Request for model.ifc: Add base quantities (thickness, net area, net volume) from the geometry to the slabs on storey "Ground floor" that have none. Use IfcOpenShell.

First a look at what the model holds.

```python
import ifcopenshell
import ifcopenshell.util.element
import ifcopenshell.util.unit

model = ifcopenshell.open("model.ifc")
print(model.schema)
for unit_type in ("LENGTHUNIT", "AREAUNIT", "VOLUMEUNIT"):
    print(unit_type, ifcopenshell.util.unit.calculate_unit_scale(model, unit_type))
storey = next(s for s in model.by_type("IfcBuildingStorey") if s.Name == "Ground floor")
slabs = [e for e in ifcopenshell.util.element.get_decomposition(storey) if e.is_a("IfcSlab")]
for e in sorted(slabs, key=lambda e: e.id()):
    print(e.id(), e.is_a(), e.Name, list(ifcopenshell.util.element.get_psets(e, qtos_only=True)), sep=" | ")
```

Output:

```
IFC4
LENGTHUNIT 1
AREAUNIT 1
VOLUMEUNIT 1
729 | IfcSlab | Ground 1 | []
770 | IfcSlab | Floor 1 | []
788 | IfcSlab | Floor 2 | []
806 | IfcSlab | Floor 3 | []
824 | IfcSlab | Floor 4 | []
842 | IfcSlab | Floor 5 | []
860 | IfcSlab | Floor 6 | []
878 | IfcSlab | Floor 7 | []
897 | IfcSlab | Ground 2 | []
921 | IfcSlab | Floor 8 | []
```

```python
import ifcopenshell
import ifcopenshell.api.pset
import ifcopenshell.geom
import ifcopenshell.util.element
import ifcopenshell.util.shape
import ifcopenshell.util.unit

model = ifcopenshell.open("model.ifc")
unit_scale = ifcopenshell.util.unit.calculate_unit_scale(model)
area_scale = ifcopenshell.util.unit.calculate_unit_scale(model, "AREAUNIT")
volume_scale = ifcopenshell.util.unit.calculate_unit_scale(model, "VOLUMEUNIT")
settings = ifcopenshell.geom.settings()

storey = next(s for s in model.by_type("IfcBuildingStorey") if s.Name == "Ground floor")
slabs = [e for e in ifcopenshell.util.element.get_decomposition(storey) if e.is_a("IfcSlab")]

for e in sorted(slabs, key=lambda e: e.id()):
    if ifcopenshell.util.element.get_psets(e, qtos_only=True, should_inherit=False):
        continue
    # Geometry comes back in metres, in the element's own axes.
    shape = ifcopenshell.geom.create_shape(settings, e)
    values = {
        "Width": ifcopenshell.util.shape.get_z(shape.geometry) / unit_scale,
        "NetArea": ifcopenshell.util.shape.get_footprint_area(shape.geometry) / area_scale,
        "NetVolume": ifcopenshell.util.shape.get_volume(shape.geometry) / volume_scale,
    }
    qto = ifcopenshell.api.pset.add_qto(model, product=e, name="Qto_SlabBaseQuantities")
    ifcopenshell.api.pset.edit_qto(model, qto=qto, properties=values)
    print(e.id(), {k: round(v, 3) for k, v in values.items()})

model.write("model_rev.ifc")
```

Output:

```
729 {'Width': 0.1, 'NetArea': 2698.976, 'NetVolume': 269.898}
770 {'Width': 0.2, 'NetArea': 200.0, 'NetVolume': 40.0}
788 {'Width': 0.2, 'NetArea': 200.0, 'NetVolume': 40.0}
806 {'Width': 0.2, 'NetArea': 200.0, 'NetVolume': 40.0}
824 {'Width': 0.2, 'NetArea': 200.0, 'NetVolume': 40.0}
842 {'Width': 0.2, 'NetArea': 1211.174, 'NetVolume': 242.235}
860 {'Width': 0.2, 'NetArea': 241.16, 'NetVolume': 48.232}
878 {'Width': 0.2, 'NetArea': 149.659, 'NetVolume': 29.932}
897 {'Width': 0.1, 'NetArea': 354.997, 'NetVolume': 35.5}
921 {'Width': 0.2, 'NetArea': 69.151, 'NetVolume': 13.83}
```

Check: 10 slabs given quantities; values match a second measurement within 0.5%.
